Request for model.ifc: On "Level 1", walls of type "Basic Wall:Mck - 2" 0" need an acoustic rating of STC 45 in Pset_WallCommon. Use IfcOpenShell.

First a look at what the model holds.

```python
import ifcopenshell
import ifcopenshell.util.element

model = ifcopenshell.open("model.ifc")
print(model.schema)
storey = next(s for s in model.by_type("IfcBuildingStorey") if s.Name == "Level 1")
walls = [e for e in ifcopenshell.util.element.get_decomposition(storey) if e.is_a("IfcWall")]
seen = {}
for e in walls:
    element_type = ifcopenshell.util.element.get_type(e)
    key = (element_type.Name if element_type != e and element_type else None, ifcopenshell.util.element.get_pset(e, "Pset_WallCommon", "AcousticRating"))
    seen[key] = seen.get(key, 0) + 1
for (name, value), count in sorted(seen.items(), key=str):
    print(count, "x", name, "|", value)
```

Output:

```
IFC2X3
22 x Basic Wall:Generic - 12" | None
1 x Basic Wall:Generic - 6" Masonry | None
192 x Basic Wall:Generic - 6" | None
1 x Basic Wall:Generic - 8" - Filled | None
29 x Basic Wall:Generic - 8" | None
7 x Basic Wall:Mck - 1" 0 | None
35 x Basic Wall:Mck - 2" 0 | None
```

```python
import ifcopenshell
import ifcopenshell.api.pset
import ifcopenshell.util.element

model = ifcopenshell.open("model.ifc")

storey = next(s for s in model.by_type("IfcBuildingStorey") if s.Name == "Level 1")
walls = [e for e in ifcopenshell.util.element.get_decomposition(storey) if e.is_a("IfcWall")]

count = 0
for e in walls:
    element_type = ifcopenshell.util.element.get_type(e)
    if element_type in (None, e) or element_type.Name != 'Basic Wall:Mck - 2" 0':
        continue
    # add_pset returns the element's existing set when there is one.
    pset = ifcopenshell.api.pset.add_pset(model, product=e, name="Pset_WallCommon")
    ifcopenshell.api.pset.edit_pset(model, pset=pset, properties={"AcousticRating": "STC 45"})
    count += 1

print(count, "walls updated")

model.write("model_updated.ifc")
```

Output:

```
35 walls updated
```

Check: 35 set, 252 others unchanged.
